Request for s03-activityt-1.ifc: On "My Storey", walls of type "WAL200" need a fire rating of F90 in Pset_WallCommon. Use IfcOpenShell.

First a look at what the model holds.

```python
import ifcopenshell
import ifcopenshell.util.element

model = ifcopenshell.open("s03-activityt-1.ifc")
print(model.schema)
storey = next(s for s in model.by_type("IfcBuildingStorey") if s.Name == "My Storey")
walls = [e for e in ifcopenshell.util.element.get_decomposition(storey) if e.is_a("IfcWall")]
seen = {}
for e in walls:
    element_type = ifcopenshell.util.element.get_type(e)
    key = (element_type.Name if element_type != e and element_type else None, ifcopenshell.util.element.get_pset(e, "Pset_WallCommon", "FireRating"))
    seen[key] = seen.get(key, 0) + 1
for (name, value), count in sorted(seen.items(), key=str):
    print(count, "x", name, "|", value)
```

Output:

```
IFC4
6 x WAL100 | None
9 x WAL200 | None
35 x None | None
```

```python
import ifcopenshell
import ifcopenshell.api.pset
import ifcopenshell.util.element

model = ifcopenshell.open("s03-activityt-1.ifc")

storey = next(s for s in model.by_type("IfcBuildingStorey") if s.Name == "My Storey")
walls = [e for e in ifcopenshell.util.element.get_decomposition(storey) if e.is_a("IfcWall")]

count = 0
for e in walls:
    element_type = ifcopenshell.util.element.get_type(e)
    if element_type in (None, e) or element_type.Name != "WAL200":
        continue
    # add_pset returns the element's existing set when there is one.
    pset = ifcopenshell.api.pset.add_pset(model, product=e, name="Pset_WallCommon")
    ifcopenshell.api.pset.edit_pset(model, pset=pset, properties={"FireRating": "F90"})
    count += 1

print(count, "walls updated")

model.write("s03-activityt-1_updated.ifc")
```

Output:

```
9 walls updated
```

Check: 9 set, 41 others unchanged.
